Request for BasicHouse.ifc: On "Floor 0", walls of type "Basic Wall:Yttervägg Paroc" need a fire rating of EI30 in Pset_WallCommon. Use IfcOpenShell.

First a look at what the model holds.

```python
import ifcopenshell
import ifcopenshell.util.element

model = ifcopenshell.open("BasicHouse.ifc")
print(model.schema)
storey = next(s for s in model.by_type("IfcBuildingStorey") if s.Name == "Floor 0")
walls = [e for e in ifcopenshell.util.element.get_decomposition(storey) if e.is_a("IfcWall")]
seen = {}
for e in walls:
    element_type = ifcopenshell.util.element.get_type(e)
    key = (element_type.Name if element_type != e and element_type else None, ifcopenshell.util.element.get_pset(e, "Pset_WallCommon", "FireRating"))
    seen[key] = seen.get(key, 0) + 1
for (name, value), count in sorted(seen.items(), key=str):
    print(count, "x", name, "|", value)
```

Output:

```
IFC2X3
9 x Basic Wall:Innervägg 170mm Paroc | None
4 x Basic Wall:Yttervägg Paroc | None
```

```python
import ifcopenshell
import ifcopenshell.api.pset
import ifcopenshell.util.element

model = ifcopenshell.open("BasicHouse.ifc")

storey = next(s for s in model.by_type("IfcBuildingStorey") if s.Name == "Floor 0")
walls = [e for e in ifcopenshell.util.element.get_decomposition(storey) if e.is_a("IfcWall")]

count = 0
for e in walls:
    element_type = ifcopenshell.util.element.get_type(e)
    if element_type in (None, e) or element_type.Name != "Basic Wall:Yttervägg Paroc":
        continue
    # add_pset returns the element's existing set when there is one.
    pset = ifcopenshell.api.pset.add_pset(model, product=e, name="Pset_WallCommon")
    ifcopenshell.api.pset.edit_pset(model, pset=pset, properties={"FireRating": "EI30"})
    count += 1

print(count, "walls updated")

model.write("BasicHouse_rev.ifc")
```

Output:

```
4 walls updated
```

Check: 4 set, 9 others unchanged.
